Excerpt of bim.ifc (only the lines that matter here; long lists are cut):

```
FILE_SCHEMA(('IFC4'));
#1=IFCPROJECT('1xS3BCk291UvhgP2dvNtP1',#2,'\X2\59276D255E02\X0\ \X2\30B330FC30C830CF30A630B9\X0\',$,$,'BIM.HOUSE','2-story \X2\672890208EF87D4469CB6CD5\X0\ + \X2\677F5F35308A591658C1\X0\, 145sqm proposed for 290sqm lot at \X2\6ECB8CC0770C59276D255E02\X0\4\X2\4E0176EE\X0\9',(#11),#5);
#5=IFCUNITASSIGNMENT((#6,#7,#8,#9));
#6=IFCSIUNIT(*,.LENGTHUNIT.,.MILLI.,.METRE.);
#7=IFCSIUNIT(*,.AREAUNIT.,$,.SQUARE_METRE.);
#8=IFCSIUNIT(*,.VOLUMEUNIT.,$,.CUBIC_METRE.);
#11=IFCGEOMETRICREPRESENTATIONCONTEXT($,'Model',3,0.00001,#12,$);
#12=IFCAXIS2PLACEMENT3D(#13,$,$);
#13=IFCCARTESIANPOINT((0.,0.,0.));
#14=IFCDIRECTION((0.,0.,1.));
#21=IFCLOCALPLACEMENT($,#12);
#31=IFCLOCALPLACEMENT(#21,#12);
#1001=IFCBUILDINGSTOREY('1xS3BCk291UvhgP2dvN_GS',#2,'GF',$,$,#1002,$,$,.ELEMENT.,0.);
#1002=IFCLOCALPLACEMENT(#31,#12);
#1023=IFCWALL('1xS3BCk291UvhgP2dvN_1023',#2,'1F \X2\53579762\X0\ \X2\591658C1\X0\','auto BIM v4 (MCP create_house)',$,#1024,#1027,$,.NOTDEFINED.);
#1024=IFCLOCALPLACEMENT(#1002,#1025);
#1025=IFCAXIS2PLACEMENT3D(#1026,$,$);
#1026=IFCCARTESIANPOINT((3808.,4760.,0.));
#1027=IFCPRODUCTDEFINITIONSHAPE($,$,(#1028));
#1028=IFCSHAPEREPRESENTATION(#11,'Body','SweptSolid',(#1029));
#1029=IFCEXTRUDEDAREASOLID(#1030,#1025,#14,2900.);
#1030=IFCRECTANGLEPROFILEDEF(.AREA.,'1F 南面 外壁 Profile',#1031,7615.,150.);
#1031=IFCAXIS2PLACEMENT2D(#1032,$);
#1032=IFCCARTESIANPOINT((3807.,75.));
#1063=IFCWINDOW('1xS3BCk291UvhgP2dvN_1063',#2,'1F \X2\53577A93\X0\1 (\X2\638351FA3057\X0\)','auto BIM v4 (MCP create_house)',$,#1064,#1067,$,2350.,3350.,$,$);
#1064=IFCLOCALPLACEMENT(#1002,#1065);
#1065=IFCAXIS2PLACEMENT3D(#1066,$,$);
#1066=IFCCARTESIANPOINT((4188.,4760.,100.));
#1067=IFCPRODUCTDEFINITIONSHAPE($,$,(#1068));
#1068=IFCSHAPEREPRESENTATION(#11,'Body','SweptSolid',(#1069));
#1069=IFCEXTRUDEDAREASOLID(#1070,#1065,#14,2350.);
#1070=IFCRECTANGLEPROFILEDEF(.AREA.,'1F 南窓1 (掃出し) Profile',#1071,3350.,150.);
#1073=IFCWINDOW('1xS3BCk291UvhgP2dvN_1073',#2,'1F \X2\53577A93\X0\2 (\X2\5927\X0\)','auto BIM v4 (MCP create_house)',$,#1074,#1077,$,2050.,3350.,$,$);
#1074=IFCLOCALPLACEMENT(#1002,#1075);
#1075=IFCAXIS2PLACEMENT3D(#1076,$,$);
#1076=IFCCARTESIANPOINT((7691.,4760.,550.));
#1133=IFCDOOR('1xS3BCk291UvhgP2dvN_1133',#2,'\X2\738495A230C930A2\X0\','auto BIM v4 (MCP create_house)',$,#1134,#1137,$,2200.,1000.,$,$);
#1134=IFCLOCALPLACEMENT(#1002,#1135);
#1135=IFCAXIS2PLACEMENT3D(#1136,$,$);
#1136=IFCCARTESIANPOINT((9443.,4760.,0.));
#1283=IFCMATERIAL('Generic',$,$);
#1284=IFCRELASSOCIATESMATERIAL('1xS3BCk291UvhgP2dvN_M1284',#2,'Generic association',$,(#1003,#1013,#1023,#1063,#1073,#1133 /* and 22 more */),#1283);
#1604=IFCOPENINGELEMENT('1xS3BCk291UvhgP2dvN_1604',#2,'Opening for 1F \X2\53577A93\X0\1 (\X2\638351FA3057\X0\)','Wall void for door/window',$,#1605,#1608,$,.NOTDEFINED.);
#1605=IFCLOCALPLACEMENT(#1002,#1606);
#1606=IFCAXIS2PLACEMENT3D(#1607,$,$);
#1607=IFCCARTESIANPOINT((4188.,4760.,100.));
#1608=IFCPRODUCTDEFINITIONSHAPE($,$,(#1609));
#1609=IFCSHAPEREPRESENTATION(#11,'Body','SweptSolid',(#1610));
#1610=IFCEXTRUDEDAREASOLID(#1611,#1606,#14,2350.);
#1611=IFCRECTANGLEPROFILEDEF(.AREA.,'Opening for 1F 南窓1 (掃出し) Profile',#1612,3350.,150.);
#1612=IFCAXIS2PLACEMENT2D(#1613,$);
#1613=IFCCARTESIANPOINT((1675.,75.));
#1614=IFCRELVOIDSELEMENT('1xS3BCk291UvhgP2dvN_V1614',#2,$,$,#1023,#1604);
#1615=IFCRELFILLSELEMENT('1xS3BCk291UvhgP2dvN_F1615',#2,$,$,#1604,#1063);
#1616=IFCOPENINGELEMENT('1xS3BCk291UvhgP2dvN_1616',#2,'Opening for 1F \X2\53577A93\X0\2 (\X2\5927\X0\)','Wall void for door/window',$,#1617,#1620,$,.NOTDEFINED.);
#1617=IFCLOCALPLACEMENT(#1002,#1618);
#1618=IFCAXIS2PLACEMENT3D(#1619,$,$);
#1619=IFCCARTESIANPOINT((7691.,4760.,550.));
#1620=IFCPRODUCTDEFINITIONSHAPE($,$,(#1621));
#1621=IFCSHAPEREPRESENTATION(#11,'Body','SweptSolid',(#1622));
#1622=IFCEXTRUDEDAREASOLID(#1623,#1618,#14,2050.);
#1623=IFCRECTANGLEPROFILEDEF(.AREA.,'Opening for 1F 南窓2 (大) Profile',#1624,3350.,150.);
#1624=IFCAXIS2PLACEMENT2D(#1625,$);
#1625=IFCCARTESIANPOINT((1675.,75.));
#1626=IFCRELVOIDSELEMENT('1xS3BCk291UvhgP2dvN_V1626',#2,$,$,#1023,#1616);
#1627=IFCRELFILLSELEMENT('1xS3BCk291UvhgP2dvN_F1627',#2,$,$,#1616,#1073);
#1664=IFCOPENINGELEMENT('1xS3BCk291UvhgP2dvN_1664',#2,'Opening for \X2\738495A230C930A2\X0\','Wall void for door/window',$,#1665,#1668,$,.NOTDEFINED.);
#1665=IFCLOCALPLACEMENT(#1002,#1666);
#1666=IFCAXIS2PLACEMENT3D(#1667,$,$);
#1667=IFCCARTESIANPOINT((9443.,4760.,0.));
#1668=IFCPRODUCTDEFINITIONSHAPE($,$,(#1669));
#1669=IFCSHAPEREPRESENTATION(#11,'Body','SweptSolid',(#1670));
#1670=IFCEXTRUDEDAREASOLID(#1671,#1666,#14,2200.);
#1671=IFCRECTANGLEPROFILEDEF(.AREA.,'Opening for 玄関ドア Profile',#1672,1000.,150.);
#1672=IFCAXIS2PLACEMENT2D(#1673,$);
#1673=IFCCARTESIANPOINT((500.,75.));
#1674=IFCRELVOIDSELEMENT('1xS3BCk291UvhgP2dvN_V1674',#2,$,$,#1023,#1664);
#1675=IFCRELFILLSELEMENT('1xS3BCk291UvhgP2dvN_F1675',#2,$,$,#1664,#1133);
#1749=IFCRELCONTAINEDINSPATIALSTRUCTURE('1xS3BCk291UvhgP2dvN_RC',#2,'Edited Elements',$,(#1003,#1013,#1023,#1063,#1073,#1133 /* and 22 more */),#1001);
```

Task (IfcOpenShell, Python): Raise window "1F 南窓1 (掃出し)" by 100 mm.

```python
import numpy as np
import ifcopenshell
import ifcopenshell.api.geometry
import ifcopenshell.util.placement
import ifcopenshell.util.unit

model = ifcopenshell.open("bim.ifc")
unit_scale = ifcopenshell.util.unit.calculate_unit_scale(model)

window = model.by_guid("1xS3BCk291UvhgP2dvN_1063")
opening = window.FillsVoids[0].RelatingOpeningElement
dz = 0.1 / unit_scale

shift = np.array([0.0, 0.0, dz])
# The window is not placed relative to its opening, so move both.
for product in (opening, window):
    matrix = ifcopenshell.util.placement.get_local_placement(product.ObjectPlacement)
    matrix[:3, 3] += shift
    ifcopenshell.api.geometry.edit_object_placement(model, product=product, matrix=matrix, is_si=False)

print(f"moved by {dz * unit_scale:+.3f} m")

model.write("bim_v2.ifc")
```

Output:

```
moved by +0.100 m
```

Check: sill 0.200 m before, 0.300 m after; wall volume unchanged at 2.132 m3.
